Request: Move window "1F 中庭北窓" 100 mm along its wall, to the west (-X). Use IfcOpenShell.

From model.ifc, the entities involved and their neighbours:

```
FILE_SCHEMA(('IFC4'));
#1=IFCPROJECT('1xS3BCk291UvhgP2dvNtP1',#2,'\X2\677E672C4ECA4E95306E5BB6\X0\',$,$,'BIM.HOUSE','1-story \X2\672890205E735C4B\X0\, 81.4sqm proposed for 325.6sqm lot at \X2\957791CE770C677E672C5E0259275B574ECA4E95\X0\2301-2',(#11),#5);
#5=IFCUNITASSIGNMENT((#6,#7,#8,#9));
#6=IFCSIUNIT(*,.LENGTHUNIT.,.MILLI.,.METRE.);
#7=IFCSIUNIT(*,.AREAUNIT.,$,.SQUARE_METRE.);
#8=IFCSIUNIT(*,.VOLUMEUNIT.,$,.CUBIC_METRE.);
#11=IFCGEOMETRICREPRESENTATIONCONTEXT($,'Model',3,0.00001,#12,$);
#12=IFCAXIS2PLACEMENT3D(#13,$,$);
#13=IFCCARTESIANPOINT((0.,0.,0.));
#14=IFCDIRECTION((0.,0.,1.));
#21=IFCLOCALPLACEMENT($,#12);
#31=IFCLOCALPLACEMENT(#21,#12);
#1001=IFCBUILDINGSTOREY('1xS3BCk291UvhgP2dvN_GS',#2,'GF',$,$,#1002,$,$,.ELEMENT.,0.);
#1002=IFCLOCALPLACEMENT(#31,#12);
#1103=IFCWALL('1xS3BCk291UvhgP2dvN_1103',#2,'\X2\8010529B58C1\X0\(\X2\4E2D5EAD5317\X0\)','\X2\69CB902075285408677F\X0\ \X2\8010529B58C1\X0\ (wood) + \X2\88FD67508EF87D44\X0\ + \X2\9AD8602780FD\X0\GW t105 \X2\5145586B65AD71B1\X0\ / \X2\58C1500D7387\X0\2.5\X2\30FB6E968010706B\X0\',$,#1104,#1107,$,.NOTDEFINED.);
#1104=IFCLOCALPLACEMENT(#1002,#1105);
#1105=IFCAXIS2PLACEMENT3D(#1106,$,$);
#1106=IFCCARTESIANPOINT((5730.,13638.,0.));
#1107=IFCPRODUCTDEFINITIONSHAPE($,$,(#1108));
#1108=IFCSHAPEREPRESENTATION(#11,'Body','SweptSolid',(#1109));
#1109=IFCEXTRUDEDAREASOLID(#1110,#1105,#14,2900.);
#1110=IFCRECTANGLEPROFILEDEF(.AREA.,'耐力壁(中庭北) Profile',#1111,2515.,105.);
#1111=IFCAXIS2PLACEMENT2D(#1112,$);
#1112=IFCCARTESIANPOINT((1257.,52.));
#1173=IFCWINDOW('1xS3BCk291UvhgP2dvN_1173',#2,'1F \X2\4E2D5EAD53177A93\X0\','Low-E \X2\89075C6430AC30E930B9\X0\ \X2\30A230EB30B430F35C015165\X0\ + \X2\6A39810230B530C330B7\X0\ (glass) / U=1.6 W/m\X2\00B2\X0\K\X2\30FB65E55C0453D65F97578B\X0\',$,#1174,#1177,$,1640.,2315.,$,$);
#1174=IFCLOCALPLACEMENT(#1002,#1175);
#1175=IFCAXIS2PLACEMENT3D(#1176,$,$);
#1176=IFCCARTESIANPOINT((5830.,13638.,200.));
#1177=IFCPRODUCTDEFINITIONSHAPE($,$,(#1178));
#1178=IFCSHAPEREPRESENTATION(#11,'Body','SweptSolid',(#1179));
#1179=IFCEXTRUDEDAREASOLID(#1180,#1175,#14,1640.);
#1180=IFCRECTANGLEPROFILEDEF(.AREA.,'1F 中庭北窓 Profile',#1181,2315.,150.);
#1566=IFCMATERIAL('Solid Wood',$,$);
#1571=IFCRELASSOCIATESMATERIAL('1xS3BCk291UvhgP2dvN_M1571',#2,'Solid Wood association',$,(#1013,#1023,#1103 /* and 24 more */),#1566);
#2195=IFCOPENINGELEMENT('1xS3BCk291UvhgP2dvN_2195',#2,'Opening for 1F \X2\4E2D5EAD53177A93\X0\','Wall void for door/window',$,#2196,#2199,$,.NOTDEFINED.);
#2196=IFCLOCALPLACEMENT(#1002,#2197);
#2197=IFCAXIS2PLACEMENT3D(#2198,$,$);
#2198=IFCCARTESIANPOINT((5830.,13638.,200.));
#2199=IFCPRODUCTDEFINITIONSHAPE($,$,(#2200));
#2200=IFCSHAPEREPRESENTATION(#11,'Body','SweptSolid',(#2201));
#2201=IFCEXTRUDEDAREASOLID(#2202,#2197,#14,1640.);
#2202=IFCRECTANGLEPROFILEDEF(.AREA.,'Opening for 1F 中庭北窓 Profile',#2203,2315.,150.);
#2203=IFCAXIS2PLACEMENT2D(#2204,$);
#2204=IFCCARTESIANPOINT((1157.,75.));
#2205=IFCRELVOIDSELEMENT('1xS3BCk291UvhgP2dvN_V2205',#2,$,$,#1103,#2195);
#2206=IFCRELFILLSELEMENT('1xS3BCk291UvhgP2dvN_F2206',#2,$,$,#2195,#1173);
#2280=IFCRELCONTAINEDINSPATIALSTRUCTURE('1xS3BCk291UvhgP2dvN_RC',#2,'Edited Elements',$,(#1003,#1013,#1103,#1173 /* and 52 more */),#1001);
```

```python
import ifcopenshell
import ifcopenshell.api.geometry
import ifcopenshell.util.placement
import ifcopenshell.util.unit

model = ifcopenshell.open("model.ifc")
unit_scale = ifcopenshell.util.unit.calculate_unit_scale(model)

window = model.by_guid("1xS3BCk291UvhgP2dvN_1173")
opening = window.FillsVoids[0].RelatingOpeningElement
wall = opening.VoidsElements[0].RelatingBuildingElement

wall_matrix = ifcopenshell.util.placement.get_local_placement(wall.ObjectPlacement)
shift = wall_matrix[:3, 0] * -0.1 / unit_scale
before = ifcopenshell.util.placement.get_local_placement(window.ObjectPlacement)[:3, 3].copy()

# The window is not placed relative to its opening, so move both.
for product in (opening, window):
    matrix = ifcopenshell.util.placement.get_local_placement(product.ObjectPlacement)
    matrix[:3, 3] += shift
    ifcopenshell.api.geometry.edit_object_placement(model, product=product, matrix=matrix, is_si=False)

after = ifcopenshell.util.placement.get_local_placement(window.ObjectPlacement)[:3, 3]
print("window moved by", (after - before).round(3) + 0.0)

model.write("model-out.ifc")
```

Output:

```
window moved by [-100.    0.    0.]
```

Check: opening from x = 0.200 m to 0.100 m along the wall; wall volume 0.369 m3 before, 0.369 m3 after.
